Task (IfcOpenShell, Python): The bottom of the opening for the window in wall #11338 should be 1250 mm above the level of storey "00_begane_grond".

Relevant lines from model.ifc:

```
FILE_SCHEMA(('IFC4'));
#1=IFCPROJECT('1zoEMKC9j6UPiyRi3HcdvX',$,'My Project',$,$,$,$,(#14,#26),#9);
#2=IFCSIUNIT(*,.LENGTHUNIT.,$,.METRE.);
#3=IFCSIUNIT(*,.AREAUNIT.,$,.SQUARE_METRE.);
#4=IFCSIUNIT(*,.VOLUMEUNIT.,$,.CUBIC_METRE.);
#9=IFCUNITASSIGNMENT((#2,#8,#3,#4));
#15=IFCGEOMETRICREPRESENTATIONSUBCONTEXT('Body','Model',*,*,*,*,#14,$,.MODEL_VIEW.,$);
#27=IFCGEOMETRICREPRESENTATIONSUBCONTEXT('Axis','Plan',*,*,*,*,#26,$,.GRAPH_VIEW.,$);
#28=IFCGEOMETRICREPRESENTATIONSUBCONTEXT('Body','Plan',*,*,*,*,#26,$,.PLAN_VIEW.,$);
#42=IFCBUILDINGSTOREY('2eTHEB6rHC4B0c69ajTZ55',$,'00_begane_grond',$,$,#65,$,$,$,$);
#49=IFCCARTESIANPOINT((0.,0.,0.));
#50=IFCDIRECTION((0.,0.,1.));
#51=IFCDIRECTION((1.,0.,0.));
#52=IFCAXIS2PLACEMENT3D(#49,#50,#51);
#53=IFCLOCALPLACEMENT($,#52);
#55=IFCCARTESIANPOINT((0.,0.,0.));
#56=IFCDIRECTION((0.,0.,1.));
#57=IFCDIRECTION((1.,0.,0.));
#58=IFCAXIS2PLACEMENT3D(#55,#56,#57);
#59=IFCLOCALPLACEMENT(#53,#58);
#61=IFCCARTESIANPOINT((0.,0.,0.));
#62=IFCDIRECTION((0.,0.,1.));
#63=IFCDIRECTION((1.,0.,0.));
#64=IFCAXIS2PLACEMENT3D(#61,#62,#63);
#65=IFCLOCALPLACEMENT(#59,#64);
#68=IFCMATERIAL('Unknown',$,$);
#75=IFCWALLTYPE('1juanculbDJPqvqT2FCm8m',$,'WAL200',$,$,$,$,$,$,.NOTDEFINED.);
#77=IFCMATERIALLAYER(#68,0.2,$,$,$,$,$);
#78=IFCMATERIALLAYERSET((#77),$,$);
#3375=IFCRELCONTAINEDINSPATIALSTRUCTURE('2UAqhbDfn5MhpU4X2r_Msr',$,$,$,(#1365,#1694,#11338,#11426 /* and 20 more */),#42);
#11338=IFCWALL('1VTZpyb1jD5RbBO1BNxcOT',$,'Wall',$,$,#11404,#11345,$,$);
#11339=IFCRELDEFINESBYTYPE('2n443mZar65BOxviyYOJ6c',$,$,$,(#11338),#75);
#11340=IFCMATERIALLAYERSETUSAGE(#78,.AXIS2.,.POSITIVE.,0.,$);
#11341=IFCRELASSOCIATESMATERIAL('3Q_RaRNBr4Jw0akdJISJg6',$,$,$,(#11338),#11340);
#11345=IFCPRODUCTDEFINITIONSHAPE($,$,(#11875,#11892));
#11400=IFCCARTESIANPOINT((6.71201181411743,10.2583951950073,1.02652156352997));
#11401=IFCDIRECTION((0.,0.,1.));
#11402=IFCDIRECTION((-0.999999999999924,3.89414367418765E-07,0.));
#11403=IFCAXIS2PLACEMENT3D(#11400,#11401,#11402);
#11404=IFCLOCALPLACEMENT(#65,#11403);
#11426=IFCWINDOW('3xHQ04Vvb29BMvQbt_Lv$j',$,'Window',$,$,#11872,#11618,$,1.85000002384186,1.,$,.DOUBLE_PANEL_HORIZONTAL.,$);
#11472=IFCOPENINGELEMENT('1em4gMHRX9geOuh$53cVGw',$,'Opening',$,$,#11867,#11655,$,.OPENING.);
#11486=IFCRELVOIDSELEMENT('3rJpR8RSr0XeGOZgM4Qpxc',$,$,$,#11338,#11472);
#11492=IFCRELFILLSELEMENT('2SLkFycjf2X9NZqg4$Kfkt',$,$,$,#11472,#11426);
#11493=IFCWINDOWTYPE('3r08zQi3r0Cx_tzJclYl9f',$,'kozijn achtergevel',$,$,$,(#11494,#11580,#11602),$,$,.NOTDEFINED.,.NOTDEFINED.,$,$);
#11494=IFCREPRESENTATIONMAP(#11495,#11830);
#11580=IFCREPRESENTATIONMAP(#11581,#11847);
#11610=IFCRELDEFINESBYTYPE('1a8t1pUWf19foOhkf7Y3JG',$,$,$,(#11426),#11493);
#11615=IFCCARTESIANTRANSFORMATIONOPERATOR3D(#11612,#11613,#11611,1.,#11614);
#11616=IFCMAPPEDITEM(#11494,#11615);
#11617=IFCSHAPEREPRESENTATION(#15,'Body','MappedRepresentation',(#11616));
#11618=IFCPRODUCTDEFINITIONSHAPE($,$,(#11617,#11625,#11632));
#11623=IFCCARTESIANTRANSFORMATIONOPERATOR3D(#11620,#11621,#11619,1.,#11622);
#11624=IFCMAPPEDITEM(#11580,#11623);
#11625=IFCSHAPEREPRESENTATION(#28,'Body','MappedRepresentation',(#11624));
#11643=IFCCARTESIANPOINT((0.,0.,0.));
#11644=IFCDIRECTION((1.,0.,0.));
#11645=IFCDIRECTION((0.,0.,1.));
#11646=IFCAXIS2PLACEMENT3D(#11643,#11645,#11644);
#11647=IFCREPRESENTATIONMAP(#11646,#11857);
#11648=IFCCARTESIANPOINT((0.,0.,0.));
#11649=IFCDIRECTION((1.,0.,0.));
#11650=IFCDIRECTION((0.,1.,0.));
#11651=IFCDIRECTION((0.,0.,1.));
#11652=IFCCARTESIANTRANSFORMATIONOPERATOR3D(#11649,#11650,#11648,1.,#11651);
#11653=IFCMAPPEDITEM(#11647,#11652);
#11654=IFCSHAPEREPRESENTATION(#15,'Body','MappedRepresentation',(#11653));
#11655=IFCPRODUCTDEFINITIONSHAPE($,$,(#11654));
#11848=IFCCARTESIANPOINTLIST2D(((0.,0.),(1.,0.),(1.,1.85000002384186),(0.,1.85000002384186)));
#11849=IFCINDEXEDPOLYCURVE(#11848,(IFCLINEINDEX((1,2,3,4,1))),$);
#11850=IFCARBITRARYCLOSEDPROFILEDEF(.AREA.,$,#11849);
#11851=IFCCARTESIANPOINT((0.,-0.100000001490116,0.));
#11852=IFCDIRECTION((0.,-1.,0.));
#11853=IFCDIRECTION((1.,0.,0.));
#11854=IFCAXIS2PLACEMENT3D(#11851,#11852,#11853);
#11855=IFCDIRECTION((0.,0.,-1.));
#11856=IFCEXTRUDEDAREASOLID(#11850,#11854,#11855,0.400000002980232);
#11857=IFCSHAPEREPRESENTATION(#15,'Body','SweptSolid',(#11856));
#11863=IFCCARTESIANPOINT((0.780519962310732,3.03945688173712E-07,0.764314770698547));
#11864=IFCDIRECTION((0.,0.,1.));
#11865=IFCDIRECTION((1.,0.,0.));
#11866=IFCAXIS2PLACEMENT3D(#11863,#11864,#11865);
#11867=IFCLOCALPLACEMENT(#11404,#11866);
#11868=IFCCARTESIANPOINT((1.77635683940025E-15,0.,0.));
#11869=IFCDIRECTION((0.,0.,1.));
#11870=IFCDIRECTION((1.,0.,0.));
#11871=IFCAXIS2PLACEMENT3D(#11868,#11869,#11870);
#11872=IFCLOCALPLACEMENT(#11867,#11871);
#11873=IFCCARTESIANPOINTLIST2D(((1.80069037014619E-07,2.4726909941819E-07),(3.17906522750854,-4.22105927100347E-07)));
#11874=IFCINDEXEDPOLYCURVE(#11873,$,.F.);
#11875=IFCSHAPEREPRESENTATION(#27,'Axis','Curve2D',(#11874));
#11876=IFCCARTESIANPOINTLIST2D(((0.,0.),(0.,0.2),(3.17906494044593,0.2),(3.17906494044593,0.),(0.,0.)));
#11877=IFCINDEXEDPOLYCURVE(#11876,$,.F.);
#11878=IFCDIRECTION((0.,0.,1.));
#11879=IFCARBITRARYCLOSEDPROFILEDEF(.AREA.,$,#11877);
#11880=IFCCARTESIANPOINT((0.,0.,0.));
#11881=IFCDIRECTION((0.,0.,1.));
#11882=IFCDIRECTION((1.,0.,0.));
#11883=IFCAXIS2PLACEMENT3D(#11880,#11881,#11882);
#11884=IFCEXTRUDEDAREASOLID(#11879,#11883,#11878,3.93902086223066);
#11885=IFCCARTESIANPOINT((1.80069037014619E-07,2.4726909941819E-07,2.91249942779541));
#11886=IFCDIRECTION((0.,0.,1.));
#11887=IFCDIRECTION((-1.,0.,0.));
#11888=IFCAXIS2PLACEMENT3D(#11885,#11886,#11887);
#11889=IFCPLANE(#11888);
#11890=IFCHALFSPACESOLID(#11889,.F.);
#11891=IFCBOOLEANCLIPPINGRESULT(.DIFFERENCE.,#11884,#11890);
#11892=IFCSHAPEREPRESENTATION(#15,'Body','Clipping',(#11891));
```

```python
import numpy as np
import ifcopenshell
import ifcopenshell.api.geometry
import ifcopenshell.geom
import ifcopenshell.util.element
import ifcopenshell.util.placement
import ifcopenshell.util.shape
import ifcopenshell.util.unit

model = ifcopenshell.open("model.ifc")
unit_scale = ifcopenshell.util.unit.calculate_unit_scale(model)

window = model.by_guid("3xHQ04Vvb29BMvQbt_Lv$j")
opening = window.FillsVoids[0].RelatingOpeningElement
storey = ifcopenshell.util.element.get_container(window, ifc_class="IfcBuildingStorey")
level = ifcopenshell.util.placement.get_local_placement(storey.ObjectPlacement)[2, 3]

# The opening's origin need not be at the sill, so measure its lowest point.
shape = ifcopenshell.geom.create_shape(ifcopenshell.geom.settings(), opening)
bottom = ifcopenshell.util.shape.get_shape_bottom_elevation(shape, shape.geometry) / unit_scale
dz = level + 1.25 / unit_scale - bottom

shift = np.array([0.0, 0.0, dz])
# The window is placed relative to its opening, so it follows when the opening moves.
matrix = ifcopenshell.util.placement.get_local_placement(opening.ObjectPlacement)
matrix[:3, 3] += shift
ifcopenshell.api.geometry.edit_object_placement(
    model, product=opening, matrix=matrix, is_si=False, should_transform_children=True
)

print(f"moved by {dz * unit_scale:+.3f} m")

model.write("model-out.ifc")
```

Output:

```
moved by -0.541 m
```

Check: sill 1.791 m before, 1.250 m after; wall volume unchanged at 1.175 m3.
